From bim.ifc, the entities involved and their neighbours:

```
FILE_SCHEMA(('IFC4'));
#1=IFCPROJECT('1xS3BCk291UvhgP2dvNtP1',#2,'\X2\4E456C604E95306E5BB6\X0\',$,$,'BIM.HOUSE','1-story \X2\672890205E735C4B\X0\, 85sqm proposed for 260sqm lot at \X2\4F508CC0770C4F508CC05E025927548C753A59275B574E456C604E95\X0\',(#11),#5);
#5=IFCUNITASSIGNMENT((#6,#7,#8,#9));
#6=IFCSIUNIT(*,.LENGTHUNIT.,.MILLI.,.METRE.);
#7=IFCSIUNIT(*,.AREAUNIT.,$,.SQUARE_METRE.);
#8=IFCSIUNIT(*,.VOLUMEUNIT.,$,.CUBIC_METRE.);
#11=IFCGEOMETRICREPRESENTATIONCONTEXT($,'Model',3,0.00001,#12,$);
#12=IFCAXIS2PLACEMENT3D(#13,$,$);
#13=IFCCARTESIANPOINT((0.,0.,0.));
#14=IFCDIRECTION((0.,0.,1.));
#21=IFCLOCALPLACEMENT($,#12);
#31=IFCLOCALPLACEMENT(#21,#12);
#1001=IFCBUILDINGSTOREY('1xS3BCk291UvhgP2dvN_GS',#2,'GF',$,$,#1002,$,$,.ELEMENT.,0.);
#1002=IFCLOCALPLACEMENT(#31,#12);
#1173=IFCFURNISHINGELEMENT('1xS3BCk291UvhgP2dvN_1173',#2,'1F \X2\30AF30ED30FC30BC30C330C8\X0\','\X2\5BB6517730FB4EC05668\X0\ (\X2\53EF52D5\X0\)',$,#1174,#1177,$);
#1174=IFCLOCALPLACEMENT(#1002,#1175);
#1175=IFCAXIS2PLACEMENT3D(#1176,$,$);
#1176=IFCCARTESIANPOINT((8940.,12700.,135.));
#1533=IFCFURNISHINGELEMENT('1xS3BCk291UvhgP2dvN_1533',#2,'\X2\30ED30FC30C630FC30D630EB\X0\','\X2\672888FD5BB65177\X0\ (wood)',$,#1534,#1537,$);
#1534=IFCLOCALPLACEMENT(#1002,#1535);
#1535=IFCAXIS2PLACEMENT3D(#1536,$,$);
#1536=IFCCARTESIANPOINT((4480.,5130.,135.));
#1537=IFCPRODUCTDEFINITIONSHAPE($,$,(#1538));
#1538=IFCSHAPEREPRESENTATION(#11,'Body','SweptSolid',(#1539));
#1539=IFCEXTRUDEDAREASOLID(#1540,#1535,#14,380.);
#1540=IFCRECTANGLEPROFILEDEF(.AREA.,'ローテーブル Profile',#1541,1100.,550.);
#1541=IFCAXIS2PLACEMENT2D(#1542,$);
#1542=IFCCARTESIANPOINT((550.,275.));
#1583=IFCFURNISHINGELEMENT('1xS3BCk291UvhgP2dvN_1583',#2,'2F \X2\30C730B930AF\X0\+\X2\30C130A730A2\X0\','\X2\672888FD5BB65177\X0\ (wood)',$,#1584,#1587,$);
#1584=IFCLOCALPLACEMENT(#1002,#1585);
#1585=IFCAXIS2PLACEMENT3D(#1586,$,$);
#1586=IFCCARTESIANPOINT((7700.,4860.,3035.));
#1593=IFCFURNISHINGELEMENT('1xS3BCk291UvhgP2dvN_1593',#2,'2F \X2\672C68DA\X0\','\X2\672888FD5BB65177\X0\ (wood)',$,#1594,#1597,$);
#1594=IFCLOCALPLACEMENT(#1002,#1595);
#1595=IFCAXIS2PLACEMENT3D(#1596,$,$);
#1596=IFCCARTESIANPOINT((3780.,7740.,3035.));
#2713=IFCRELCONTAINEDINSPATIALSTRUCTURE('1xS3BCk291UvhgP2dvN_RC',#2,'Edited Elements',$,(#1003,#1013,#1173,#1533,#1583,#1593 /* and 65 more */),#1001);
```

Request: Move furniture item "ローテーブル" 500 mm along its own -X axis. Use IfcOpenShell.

```python
import ifcopenshell
import ifcopenshell.api.geometry
import ifcopenshell.util.placement

model = ifcopenshell.open("bim.ifc")

item = model.by_guid("1xS3BCk291UvhgP2dvN_1533")
matrix = ifcopenshell.util.placement.get_local_placement(item.ObjectPlacement)
matrix[:3, 3] -= matrix[:3, 0] * 500.0
ifcopenshell.api.geometry.edit_object_placement(model, product=item, matrix=matrix, is_si=False)

print(ifcopenshell.util.placement.get_local_placement(item.ObjectPlacement).round(3) + 0.0)

model.write("bim_updated.ifc")
```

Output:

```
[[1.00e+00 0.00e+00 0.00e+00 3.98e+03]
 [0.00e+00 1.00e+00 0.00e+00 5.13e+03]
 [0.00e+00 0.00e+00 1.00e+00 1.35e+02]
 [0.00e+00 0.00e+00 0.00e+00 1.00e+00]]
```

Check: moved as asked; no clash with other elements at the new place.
